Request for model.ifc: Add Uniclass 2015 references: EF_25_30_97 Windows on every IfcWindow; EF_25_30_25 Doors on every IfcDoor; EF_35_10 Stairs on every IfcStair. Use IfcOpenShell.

First a look at what the model holds.

```python
import ifcopenshell

model = ifcopenshell.open("model.ifc")
print(model.schema)
print("classifications:", [c.Name for c in model.by_type("IfcClassification")])
for ifc_class in ("IfcDoor", "IfcRoof", "IfcStair", "IfcWall", "IfcWindow"):
    print(ifc_class, len(model.by_type(ifc_class)))
```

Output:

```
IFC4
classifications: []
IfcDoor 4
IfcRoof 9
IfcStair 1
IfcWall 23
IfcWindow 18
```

```python
import ifcopenshell
import ifcopenshell.api.classification

model = ifcopenshell.open("model.ifc")

system = ifcopenshell.api.classification.add_classification(model, classification="Uniclass 2015")

codes = {
    "IfcWindow": ("EF_25_30_97", "Windows"),
    "IfcDoor": ("EF_25_30_25", "Doors"),
    "IfcStair": ("EF_35_10", "Stairs"),
}
for ifc_class, (code, name) in codes.items():
    products = model.by_type(ifc_class)
    ifcopenshell.api.classification.add_reference(
        model, products=products, classification=system, identification=code, name=name
    )
    print(code, len(products))

model.write("model_v2.ifc")
```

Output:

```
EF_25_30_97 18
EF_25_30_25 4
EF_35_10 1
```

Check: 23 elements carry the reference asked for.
